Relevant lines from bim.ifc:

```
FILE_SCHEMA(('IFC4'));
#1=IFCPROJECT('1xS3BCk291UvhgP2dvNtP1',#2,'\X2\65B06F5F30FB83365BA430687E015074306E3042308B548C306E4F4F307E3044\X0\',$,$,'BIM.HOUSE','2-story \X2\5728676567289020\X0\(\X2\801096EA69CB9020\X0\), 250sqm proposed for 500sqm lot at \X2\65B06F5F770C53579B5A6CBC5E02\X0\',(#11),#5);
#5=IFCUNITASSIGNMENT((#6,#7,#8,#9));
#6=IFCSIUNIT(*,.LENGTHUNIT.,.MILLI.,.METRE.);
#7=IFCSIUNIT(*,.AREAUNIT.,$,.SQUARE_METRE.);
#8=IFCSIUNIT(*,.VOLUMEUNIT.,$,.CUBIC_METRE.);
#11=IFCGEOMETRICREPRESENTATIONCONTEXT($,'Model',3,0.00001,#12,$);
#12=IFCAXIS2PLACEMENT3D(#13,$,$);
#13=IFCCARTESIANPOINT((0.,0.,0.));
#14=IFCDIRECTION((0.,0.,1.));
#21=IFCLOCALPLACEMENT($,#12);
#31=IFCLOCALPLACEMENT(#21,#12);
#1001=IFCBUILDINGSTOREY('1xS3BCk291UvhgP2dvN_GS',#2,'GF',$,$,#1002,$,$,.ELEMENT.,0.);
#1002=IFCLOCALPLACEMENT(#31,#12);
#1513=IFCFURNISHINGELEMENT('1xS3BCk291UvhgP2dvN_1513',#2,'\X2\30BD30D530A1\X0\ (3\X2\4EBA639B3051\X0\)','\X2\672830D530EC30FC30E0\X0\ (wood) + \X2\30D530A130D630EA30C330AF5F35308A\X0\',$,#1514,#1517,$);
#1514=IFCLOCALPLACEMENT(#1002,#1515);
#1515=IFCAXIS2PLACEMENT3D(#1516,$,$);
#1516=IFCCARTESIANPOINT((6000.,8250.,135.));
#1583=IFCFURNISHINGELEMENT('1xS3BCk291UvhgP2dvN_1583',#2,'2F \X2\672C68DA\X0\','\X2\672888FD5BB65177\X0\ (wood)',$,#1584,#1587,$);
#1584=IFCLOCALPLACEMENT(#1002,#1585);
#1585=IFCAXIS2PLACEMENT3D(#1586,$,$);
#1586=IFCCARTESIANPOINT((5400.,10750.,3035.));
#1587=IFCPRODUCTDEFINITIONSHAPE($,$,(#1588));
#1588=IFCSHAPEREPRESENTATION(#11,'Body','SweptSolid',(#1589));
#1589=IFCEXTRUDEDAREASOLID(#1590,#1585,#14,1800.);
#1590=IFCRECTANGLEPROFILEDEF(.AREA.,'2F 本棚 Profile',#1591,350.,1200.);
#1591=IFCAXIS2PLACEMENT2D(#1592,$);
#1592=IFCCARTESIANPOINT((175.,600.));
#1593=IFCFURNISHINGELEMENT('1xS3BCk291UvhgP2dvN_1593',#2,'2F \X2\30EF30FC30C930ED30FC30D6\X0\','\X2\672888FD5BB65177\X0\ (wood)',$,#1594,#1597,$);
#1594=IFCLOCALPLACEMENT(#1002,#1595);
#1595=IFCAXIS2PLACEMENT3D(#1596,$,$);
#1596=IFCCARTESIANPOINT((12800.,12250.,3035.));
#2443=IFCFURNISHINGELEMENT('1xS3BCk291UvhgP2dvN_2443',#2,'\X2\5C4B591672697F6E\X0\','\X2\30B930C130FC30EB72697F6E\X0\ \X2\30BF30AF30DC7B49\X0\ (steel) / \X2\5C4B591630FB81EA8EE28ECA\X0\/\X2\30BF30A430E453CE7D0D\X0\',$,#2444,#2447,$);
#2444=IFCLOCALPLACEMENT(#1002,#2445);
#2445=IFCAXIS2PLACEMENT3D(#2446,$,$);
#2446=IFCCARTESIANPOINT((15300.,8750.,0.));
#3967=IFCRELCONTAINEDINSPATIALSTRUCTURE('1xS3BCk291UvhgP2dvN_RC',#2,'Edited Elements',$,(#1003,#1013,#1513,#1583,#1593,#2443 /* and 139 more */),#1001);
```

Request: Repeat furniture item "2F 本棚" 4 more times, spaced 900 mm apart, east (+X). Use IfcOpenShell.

```python
import numpy as np
import ifcopenshell
import ifcopenshell.api.geometry
import ifcopenshell.api.root
import ifcopenshell.util.element
import ifcopenshell.util.placement
import ifcopenshell.util.unit

model = ifcopenshell.open("bim.ifc")
unit_scale = ifcopenshell.util.unit.calculate_unit_scale(model)


def reuse_history(source, copy):
    """copy_class also copies each property set's owner history, people and application; keep the originals."""
    for rel in copy.IsDefinedBy:
        if rel.is_a("IfcRelDefinesByProperties") and (history := rel.RelatingPropertyDefinition.OwnerHistory):
            rel.RelatingPropertyDefinition.OwnerHistory = source.OwnerHistory
            ifcopenshell.util.element.remove_deep2(model, history)


source = model.by_guid("1xS3BCk291UvhgP2dvN_1583")
base = ifcopenshell.util.placement.get_local_placement(source.ObjectPlacement)
step = np.array([1.0, 0.0, 0.0]) * 0.9 / unit_scale

for i in range(1, 5):
    copy = ifcopenshell.api.root.copy_class(model, product=source)
    copy.Representation = ifcopenshell.util.element.copy_deep(
        model, source.Representation, exclude=["IfcGeometricRepresentationContext", "IfcRepresentationMap"]
    )
    reuse_history(source, copy)
    matrix = base.copy()
    matrix[:3, 3] += i * step
    print("added at", matrix[:3, 3].round(3) + 0.0)
    ifcopenshell.api.geometry.edit_object_placement(model, product=copy, matrix=matrix, is_si=False)

model.write("bim_rev.ifc")
```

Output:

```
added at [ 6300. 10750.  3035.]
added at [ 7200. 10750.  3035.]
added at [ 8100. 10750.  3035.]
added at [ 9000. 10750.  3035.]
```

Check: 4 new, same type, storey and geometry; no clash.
